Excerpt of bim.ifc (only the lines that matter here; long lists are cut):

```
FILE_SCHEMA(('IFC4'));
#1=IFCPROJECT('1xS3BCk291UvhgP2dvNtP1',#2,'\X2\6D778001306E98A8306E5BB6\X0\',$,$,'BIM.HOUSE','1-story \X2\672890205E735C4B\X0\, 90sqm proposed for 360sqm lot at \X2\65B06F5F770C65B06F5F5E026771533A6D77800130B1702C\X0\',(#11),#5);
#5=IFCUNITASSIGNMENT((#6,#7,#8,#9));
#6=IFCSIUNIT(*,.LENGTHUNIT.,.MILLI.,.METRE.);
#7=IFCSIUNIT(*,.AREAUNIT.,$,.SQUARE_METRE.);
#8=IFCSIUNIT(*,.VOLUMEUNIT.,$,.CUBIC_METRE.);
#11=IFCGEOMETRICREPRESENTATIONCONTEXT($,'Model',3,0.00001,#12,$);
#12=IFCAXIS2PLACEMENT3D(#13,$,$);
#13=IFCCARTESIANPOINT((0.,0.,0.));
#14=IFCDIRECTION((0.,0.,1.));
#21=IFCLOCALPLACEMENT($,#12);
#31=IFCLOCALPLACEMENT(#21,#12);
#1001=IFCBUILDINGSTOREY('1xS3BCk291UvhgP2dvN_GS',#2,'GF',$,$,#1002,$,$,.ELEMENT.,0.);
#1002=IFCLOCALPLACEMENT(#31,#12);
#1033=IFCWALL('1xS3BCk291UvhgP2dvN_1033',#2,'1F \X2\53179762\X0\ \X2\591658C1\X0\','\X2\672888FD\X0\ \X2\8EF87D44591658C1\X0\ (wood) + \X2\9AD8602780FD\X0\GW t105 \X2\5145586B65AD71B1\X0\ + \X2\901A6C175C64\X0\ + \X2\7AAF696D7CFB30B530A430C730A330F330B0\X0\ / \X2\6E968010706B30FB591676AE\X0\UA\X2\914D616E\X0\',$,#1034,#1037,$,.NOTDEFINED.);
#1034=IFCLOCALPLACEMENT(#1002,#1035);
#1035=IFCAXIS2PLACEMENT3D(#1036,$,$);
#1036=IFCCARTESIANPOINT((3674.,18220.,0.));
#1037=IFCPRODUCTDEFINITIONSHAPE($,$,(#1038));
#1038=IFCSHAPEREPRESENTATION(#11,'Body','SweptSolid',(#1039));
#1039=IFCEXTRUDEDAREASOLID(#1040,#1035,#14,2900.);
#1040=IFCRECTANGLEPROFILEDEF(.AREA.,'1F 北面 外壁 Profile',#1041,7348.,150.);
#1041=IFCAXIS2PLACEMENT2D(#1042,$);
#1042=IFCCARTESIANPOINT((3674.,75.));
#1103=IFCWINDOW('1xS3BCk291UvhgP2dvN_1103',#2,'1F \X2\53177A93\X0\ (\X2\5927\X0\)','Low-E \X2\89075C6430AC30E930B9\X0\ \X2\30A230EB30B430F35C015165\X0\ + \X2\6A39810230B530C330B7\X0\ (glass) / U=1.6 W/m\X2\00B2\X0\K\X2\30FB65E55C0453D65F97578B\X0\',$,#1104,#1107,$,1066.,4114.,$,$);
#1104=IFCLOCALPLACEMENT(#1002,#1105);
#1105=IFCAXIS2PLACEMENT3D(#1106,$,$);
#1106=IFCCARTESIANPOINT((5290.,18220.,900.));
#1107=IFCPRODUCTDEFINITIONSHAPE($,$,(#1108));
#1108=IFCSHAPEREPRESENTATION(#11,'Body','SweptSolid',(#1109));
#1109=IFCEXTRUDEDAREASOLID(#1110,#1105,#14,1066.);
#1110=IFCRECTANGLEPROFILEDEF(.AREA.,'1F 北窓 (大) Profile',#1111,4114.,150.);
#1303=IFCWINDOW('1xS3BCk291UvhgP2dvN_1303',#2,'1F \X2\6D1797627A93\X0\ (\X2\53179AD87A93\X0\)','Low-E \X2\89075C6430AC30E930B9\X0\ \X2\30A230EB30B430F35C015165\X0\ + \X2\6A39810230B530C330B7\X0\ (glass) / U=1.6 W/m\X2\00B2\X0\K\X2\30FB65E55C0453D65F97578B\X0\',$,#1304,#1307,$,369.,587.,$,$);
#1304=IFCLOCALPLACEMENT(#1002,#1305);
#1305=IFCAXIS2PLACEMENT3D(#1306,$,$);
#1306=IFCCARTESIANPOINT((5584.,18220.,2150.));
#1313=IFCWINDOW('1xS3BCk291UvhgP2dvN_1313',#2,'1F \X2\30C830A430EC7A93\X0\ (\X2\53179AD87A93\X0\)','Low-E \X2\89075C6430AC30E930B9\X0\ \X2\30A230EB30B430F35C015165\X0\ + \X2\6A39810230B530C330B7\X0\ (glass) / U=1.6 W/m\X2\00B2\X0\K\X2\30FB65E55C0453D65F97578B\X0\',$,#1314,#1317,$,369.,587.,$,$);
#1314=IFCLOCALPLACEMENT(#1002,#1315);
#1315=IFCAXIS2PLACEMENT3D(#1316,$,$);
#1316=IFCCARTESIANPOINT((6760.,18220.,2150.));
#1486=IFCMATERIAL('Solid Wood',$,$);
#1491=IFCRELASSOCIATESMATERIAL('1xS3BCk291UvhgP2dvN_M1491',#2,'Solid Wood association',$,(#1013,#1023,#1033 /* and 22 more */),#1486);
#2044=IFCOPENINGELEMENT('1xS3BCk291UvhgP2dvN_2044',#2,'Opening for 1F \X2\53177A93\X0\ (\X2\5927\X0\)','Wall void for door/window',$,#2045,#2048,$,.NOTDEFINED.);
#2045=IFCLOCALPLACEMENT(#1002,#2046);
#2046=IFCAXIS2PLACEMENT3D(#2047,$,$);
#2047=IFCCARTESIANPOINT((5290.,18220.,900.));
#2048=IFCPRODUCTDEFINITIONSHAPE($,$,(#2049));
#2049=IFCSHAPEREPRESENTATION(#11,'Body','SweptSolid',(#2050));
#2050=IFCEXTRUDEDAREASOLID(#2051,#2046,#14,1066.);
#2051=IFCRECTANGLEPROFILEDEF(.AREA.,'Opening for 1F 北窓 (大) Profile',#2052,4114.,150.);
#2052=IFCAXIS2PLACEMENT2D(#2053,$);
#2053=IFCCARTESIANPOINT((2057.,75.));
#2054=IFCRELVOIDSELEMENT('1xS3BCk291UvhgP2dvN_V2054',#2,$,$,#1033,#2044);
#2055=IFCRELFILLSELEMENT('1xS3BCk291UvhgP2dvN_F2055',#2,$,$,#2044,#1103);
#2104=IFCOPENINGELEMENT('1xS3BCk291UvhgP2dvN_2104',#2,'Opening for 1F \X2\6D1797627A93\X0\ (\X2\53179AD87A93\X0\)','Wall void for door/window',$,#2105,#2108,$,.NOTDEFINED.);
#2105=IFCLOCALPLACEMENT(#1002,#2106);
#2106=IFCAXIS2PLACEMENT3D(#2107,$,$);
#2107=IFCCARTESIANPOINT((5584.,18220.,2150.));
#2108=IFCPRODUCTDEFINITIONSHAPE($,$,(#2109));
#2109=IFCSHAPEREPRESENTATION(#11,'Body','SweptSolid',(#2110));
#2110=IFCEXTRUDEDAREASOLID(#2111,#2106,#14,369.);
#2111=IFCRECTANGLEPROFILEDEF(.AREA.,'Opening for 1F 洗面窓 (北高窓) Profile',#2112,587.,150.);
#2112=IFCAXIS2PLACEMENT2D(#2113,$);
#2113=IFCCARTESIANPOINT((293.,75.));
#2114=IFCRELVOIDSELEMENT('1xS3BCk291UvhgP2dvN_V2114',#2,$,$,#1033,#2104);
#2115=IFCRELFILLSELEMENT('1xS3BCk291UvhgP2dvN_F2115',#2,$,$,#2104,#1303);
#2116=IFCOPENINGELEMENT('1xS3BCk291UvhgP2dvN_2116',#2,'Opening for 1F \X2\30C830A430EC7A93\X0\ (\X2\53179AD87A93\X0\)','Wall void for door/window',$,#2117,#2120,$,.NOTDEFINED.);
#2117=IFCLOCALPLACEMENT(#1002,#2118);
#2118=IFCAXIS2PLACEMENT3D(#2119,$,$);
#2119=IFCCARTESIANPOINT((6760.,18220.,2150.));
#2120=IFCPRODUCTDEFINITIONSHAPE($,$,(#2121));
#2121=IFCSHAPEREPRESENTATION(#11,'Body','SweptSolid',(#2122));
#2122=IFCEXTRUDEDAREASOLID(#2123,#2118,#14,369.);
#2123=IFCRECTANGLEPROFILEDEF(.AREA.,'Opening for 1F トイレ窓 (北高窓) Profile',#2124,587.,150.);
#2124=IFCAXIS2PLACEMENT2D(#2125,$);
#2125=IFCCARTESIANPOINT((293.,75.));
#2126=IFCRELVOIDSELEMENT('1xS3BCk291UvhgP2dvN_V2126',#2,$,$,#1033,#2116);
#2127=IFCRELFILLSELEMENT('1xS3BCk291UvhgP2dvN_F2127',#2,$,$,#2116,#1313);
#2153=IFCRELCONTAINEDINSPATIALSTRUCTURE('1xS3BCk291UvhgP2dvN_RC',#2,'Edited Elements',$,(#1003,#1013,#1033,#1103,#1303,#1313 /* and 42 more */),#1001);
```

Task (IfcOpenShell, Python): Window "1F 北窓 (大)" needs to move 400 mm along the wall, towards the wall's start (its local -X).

```python
import ifcopenshell
import ifcopenshell.api.geometry
import ifcopenshell.util.placement

model = ifcopenshell.open("bim.ifc")

window = model.by_guid("1xS3BCk291UvhgP2dvN_1103")
opening = window.FillsVoids[0].RelatingOpeningElement
wall = opening.VoidsElements[0].RelatingBuildingElement

wall_matrix = ifcopenshell.util.placement.get_local_placement(wall.ObjectPlacement)
shift = wall_matrix[:3, 0] * -400.0
before = ifcopenshell.util.placement.get_local_placement(window.ObjectPlacement)[:3, 3].copy()

# The window is not placed relative to its opening, so move both.
for product in (opening, window):
    matrix = ifcopenshell.util.placement.get_local_placement(product.ObjectPlacement)
    matrix[:3, 3] += shift
    ifcopenshell.api.geometry.edit_object_placement(model, product=product, matrix=matrix, is_si=False)

after = ifcopenshell.util.placement.get_local_placement(window.ObjectPlacement)[:3, 3]
print("window moved by", (after - before).round(3) + 0.0)

model.write("bim_v2.ifc")
```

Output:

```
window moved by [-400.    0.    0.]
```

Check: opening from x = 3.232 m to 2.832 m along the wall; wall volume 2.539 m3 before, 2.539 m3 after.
